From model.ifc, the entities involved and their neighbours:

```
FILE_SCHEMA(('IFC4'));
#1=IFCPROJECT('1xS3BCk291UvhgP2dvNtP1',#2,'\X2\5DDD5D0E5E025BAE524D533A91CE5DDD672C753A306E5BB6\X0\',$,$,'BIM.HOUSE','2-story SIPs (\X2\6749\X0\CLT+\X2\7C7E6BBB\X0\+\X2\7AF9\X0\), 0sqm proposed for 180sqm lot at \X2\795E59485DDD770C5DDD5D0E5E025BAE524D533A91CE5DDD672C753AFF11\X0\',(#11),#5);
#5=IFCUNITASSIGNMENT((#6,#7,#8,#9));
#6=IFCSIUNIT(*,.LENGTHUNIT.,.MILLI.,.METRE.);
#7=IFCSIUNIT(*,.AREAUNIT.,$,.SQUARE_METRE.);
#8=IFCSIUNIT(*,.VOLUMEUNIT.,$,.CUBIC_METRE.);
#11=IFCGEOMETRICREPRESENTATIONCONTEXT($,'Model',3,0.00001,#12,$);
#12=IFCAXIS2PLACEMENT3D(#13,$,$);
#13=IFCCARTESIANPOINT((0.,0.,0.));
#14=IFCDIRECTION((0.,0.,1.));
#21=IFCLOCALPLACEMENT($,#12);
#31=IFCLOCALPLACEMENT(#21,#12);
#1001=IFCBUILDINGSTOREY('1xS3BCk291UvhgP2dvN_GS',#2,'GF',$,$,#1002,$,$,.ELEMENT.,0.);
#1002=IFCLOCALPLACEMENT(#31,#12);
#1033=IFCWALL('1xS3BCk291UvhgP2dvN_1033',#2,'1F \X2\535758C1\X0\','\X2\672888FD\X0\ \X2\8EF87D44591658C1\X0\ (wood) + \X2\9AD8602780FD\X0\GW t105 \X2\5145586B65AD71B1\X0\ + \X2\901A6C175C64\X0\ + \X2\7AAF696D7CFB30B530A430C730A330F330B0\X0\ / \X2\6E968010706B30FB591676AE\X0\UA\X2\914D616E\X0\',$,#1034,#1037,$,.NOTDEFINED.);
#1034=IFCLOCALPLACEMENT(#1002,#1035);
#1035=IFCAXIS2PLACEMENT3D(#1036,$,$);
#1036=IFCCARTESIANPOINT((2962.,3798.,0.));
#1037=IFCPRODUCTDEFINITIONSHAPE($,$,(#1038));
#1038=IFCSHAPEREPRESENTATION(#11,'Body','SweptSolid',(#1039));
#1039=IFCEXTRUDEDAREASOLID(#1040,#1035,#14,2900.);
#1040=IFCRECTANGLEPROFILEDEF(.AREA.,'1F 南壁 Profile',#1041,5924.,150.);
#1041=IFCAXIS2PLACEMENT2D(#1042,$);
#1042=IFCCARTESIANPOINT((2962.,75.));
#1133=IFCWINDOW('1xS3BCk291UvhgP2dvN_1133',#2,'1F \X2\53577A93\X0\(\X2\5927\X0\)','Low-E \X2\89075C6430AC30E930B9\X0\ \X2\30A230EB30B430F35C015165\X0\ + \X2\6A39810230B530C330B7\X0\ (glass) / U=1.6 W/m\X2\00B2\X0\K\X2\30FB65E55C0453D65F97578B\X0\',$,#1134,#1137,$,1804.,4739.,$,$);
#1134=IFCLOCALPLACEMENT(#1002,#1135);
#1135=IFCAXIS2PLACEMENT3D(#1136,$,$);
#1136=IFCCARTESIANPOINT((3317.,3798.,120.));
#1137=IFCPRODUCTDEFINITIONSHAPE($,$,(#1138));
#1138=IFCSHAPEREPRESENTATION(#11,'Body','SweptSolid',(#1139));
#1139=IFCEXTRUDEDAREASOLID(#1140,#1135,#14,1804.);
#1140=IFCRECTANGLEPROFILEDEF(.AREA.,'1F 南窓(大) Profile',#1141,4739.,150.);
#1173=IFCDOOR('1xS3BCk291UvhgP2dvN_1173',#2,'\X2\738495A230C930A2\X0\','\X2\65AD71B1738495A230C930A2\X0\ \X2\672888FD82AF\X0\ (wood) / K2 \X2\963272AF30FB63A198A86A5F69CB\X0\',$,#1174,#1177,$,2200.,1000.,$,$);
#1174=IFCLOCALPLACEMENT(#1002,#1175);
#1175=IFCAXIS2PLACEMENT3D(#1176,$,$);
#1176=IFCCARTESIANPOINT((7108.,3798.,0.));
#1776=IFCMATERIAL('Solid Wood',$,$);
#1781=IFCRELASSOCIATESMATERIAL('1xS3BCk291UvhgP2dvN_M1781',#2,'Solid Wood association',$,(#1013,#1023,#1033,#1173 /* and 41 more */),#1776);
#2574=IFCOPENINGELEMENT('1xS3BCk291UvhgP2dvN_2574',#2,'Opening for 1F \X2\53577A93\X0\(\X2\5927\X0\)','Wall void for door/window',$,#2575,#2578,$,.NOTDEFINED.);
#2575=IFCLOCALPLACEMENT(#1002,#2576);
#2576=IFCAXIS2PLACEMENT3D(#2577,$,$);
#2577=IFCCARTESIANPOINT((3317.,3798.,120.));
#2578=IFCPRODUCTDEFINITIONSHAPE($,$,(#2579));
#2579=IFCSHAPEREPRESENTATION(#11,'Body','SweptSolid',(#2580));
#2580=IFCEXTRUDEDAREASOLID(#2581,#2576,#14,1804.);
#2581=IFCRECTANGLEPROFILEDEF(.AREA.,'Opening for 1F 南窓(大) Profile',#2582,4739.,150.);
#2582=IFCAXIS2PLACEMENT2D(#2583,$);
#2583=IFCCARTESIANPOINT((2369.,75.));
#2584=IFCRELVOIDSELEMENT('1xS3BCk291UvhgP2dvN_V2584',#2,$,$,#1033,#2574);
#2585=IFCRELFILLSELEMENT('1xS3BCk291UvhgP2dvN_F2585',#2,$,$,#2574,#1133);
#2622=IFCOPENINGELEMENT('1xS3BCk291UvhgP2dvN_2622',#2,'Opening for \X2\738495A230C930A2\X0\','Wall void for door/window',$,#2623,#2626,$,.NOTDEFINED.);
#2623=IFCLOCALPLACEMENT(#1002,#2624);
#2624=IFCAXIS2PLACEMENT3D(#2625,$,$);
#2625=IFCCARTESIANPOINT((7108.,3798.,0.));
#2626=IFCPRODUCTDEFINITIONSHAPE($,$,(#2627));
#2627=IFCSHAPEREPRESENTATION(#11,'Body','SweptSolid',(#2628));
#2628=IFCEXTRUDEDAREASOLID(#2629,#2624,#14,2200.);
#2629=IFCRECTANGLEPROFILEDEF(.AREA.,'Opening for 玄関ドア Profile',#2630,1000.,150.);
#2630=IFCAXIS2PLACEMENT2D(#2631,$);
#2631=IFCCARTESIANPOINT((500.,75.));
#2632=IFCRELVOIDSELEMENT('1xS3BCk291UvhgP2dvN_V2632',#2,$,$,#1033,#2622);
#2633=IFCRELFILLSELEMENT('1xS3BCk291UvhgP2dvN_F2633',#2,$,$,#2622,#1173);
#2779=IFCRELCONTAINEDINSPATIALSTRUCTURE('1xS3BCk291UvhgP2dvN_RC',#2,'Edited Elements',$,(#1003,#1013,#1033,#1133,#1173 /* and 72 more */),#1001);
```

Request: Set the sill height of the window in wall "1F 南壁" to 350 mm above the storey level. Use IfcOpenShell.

```python
import numpy as np
import ifcopenshell
import ifcopenshell.api.geometry
import ifcopenshell.geom
import ifcopenshell.util.element
import ifcopenshell.util.placement
import ifcopenshell.util.shape
import ifcopenshell.util.unit

model = ifcopenshell.open("model.ifc")
unit_scale = ifcopenshell.util.unit.calculate_unit_scale(model)

window = model.by_guid("1xS3BCk291UvhgP2dvN_1133")
opening = window.FillsVoids[0].RelatingOpeningElement
storey = ifcopenshell.util.element.get_container(window, ifc_class="IfcBuildingStorey")
level = ifcopenshell.util.placement.get_local_placement(storey.ObjectPlacement)[2, 3]

# The opening's origin need not be at the sill, so measure its lowest point.
shape = ifcopenshell.geom.create_shape(ifcopenshell.geom.settings(), opening)
bottom = ifcopenshell.util.shape.get_shape_bottom_elevation(shape, shape.geometry) / unit_scale
dz = level + 0.35 / unit_scale - bottom

shift = np.array([0.0, 0.0, dz])
# The window is not placed relative to its opening, so move both.
for product in (opening, window):
    matrix = ifcopenshell.util.placement.get_local_placement(product.ObjectPlacement)
    matrix[:3, 3] += shift
    ifcopenshell.api.geometry.edit_object_placement(model, product=product, matrix=matrix, is_si=False)

print(f"moved by {dz * unit_scale:+.3f} m")

model.write("model-out.ifc")
```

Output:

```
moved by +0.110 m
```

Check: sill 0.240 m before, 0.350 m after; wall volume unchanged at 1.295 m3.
